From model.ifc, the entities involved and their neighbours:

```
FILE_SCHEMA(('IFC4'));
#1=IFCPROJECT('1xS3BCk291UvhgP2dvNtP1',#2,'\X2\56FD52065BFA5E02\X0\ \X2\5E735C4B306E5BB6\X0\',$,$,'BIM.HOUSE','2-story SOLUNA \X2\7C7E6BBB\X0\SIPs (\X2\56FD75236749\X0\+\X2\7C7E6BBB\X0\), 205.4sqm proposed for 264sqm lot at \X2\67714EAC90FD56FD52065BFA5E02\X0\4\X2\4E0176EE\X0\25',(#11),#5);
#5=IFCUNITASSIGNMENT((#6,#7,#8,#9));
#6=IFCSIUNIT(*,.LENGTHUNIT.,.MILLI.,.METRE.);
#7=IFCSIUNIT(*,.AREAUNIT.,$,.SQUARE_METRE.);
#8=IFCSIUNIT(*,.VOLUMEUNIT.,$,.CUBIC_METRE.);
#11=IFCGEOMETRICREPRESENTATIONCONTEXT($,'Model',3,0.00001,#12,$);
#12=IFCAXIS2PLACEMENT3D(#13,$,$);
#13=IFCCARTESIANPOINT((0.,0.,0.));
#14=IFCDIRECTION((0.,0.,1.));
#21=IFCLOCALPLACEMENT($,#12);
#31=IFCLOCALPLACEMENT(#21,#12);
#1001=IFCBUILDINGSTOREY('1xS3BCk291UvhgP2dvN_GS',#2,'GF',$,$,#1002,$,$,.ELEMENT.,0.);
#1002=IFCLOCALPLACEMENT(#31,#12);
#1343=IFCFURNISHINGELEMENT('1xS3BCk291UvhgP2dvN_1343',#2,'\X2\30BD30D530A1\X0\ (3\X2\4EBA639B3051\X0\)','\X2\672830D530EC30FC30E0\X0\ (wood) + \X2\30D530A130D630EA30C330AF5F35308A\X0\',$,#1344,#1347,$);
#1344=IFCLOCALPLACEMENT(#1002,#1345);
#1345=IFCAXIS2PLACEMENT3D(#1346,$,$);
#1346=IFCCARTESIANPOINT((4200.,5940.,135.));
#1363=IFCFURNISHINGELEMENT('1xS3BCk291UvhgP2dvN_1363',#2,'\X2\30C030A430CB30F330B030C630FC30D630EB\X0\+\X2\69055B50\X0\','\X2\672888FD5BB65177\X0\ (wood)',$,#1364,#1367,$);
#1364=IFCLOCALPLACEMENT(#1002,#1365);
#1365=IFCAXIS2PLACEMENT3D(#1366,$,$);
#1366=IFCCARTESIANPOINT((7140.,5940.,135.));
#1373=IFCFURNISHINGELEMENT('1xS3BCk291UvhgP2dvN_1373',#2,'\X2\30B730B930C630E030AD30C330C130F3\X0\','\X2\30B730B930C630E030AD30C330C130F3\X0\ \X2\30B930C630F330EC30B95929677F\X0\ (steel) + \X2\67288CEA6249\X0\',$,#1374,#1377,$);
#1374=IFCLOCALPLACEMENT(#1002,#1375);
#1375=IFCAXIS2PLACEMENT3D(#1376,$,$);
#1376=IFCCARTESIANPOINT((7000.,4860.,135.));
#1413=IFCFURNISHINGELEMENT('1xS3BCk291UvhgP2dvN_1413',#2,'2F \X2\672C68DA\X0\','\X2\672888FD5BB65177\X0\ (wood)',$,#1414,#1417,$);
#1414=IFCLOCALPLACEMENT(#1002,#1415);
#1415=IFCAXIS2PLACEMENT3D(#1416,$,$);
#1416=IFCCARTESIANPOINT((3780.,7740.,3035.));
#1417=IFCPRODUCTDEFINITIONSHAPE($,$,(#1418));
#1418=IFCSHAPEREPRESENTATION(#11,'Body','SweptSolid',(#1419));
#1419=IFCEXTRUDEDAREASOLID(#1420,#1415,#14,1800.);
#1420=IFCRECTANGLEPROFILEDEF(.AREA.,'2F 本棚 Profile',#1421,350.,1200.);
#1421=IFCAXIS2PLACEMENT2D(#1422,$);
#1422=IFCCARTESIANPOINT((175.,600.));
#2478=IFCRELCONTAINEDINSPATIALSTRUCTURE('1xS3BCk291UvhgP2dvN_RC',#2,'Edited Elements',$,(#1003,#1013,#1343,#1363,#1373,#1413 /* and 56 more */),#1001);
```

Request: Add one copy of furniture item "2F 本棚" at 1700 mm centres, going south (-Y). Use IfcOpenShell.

```python
import numpy as np
import ifcopenshell
import ifcopenshell.api.geometry
import ifcopenshell.api.root
import ifcopenshell.util.element
import ifcopenshell.util.placement

model = ifcopenshell.open("model.ifc")


def reuse_history(source, copy):
    """copy_class also copies each property set's owner history, people and application; keep the originals."""
    for rel in copy.IsDefinedBy:
        if rel.is_a("IfcRelDefinesByProperties") and (history := rel.RelatingPropertyDefinition.OwnerHistory):
            rel.RelatingPropertyDefinition.OwnerHistory = source.OwnerHistory
            ifcopenshell.util.element.remove_deep2(model, history)


source = model.by_id(1413)
base = ifcopenshell.util.placement.get_local_placement(source.ObjectPlacement)
step = np.array([0.0, -1.0, 0.0]) * 1700.0

for i in range(1, 2):
    copy = ifcopenshell.api.root.copy_class(model, product=source)
    copy.Representation = ifcopenshell.util.element.copy_deep(
        model, source.Representation, exclude=["IfcGeometricRepresentationContext", "IfcRepresentationMap"]
    )
    reuse_history(source, copy)
    matrix = base.copy()
    matrix[:3, 3] += i * step
    print("added at", matrix[:3, 3].round(3) + 0.0)
    ifcopenshell.api.geometry.edit_object_placement(model, product=copy, matrix=matrix, is_si=False)

model.write("model_v2.ifc")
```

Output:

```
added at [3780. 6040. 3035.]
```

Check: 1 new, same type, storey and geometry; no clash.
